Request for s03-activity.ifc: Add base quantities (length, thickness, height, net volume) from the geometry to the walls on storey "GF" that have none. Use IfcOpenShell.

First a look at what the model holds.

```python
import ifcopenshell
import ifcopenshell.util.element
import ifcopenshell.util.unit

model = ifcopenshell.open("s03-activity.ifc")
print(model.schema)
for unit_type in ("LENGTHUNIT", "AREAUNIT", "VOLUMEUNIT"):
    print(unit_type, ifcopenshell.util.unit.calculate_unit_scale(model, unit_type))
storey = next(s for s in model.by_type("IfcBuildingStorey") if s.Name == "GF")
walls = [e for e in ifcopenshell.util.element.get_decomposition(storey) if e.is_a("IfcWall")]
for e in sorted(walls, key=lambda e: e.id()):
    print(e.id(), e.is_a(), e.Name, list(ifcopenshell.util.element.get_psets(e, qtos_only=True)), sep=" | ")
```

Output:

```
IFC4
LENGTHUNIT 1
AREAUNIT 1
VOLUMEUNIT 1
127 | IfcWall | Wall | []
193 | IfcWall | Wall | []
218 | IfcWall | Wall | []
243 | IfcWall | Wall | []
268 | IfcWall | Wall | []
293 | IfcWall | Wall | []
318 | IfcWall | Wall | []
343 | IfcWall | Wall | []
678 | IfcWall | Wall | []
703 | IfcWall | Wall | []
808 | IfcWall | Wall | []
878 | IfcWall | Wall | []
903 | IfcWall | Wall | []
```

```python
import ifcopenshell
import ifcopenshell.api.pset
import ifcopenshell.geom
import ifcopenshell.util.element
import ifcopenshell.util.shape
import ifcopenshell.util.unit

model = ifcopenshell.open("s03-activity.ifc")
unit_scale = ifcopenshell.util.unit.calculate_unit_scale(model)
volume_scale = ifcopenshell.util.unit.calculate_unit_scale(model, "VOLUMEUNIT")
settings = ifcopenshell.geom.settings()

storey = next(s for s in model.by_type("IfcBuildingStorey") if s.Name == "GF")
walls = [e for e in ifcopenshell.util.element.get_decomposition(storey) if e.is_a("IfcWall")]

for e in sorted(walls, key=lambda e: e.id()):
    if ifcopenshell.util.element.get_psets(e, qtos_only=True, should_inherit=False):
        continue
    # Geometry comes back in metres, in the element's own axes.
    shape = ifcopenshell.geom.create_shape(settings, e)
    values = {
        "Length": ifcopenshell.util.shape.get_x(shape.geometry) / unit_scale,
        "Width": ifcopenshell.util.shape.get_y(shape.geometry) / unit_scale,
        "Height": ifcopenshell.util.shape.get_z(shape.geometry) / unit_scale,
        "NetVolume": ifcopenshell.util.shape.get_volume(shape.geometry) / volume_scale,
    }
    qto = ifcopenshell.api.pset.add_qto(model, product=e, name="Qto_WallBaseQuantities")
    ifcopenshell.api.pset.edit_qto(model, qto=qto, properties=values)
    print(e.id(), {k: round(v, 3) for k, v in values.items()})

model.write("s03-activity_rev.ifc")
```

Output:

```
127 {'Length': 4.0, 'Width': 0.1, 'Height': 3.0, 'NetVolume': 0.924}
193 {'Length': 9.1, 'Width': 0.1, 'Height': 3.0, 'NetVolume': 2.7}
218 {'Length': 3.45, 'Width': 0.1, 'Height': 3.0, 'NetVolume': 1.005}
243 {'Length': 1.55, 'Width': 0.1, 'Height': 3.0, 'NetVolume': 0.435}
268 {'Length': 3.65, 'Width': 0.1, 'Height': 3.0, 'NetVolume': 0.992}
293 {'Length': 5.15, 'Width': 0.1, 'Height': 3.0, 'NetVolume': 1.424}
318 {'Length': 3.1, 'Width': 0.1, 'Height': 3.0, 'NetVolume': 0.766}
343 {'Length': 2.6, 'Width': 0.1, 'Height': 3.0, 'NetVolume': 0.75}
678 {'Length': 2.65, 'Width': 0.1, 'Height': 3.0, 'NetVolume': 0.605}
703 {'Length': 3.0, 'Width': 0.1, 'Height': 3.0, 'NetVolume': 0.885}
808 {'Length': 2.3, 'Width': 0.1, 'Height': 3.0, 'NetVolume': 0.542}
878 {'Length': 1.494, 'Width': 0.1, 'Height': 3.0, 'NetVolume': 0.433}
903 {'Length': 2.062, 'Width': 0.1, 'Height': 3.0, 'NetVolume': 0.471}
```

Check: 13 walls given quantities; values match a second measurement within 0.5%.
